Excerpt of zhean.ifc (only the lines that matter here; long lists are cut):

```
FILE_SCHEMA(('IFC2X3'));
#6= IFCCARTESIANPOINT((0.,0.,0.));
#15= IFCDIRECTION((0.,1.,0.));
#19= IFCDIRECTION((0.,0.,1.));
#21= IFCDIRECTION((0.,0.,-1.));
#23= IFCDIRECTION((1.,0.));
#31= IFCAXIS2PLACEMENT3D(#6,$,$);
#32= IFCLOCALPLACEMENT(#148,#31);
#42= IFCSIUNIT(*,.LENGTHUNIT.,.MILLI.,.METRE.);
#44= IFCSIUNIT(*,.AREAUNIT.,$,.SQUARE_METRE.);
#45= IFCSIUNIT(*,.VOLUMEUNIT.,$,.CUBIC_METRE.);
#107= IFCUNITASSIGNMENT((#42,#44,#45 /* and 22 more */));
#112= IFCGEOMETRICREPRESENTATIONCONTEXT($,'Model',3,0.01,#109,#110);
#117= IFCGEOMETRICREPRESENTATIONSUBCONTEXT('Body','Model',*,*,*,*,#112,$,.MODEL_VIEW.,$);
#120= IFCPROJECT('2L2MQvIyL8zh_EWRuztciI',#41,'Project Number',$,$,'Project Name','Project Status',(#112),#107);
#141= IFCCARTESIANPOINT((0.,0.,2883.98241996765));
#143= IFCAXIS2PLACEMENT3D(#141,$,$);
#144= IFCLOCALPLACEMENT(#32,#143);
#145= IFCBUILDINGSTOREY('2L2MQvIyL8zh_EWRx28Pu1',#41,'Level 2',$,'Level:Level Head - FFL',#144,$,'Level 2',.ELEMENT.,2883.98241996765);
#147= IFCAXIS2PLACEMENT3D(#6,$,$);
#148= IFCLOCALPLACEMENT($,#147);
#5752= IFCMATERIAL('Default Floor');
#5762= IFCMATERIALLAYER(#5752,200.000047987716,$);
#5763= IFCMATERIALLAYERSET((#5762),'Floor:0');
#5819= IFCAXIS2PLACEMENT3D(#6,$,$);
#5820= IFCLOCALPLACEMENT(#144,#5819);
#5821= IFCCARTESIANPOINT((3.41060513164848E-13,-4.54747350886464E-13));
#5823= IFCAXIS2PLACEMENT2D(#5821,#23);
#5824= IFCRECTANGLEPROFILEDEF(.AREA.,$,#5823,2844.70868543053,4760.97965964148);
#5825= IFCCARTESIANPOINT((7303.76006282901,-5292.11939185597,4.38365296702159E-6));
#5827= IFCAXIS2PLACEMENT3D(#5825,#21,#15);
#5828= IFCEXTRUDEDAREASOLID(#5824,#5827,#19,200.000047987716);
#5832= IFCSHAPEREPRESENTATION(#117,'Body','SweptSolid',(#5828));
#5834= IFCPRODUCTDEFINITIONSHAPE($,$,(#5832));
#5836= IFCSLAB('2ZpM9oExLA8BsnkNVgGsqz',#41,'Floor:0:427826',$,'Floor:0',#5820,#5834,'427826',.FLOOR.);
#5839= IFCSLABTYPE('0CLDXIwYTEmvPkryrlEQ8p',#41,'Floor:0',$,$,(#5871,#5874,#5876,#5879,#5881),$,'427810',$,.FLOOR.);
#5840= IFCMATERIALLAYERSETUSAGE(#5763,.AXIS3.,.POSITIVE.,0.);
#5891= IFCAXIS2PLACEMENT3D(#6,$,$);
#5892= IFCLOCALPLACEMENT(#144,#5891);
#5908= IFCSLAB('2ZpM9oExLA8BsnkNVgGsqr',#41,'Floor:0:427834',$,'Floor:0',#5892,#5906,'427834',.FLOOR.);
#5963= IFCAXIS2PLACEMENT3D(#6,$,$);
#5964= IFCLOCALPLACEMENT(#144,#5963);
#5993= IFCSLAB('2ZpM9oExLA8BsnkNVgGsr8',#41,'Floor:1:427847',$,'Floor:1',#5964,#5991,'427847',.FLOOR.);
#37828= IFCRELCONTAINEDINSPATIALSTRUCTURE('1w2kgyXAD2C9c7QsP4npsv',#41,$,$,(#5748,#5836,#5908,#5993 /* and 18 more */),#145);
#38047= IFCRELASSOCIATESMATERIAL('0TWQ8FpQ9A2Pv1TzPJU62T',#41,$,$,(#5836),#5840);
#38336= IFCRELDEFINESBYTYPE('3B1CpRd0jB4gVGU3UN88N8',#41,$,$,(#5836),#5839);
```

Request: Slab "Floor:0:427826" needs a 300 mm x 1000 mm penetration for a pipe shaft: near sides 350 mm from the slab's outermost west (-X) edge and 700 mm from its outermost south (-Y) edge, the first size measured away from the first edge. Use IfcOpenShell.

```python
import numpy as np
import ifcopenshell
import ifcopenshell.api.feature
import ifcopenshell.api.geometry
import ifcopenshell.api.root
import ifcopenshell.geom
import ifcopenshell.util.placement
import ifcopenshell.util.representation
import ifcopenshell.util.shape
import ifcopenshell.util.unit

model = ifcopenshell.open("zhean.ifc")
unit_scale = ifcopenshell.util.unit.calculate_unit_scale(model)
settings = ifcopenshell.geom.settings()


def volume(element):
    """Net volume in cubic metres, openings subtracted."""
    shape = ifcopenshell.geom.create_shape(settings, element)
    return ifcopenshell.util.shape.get_volume(shape.geometry)


slab = model.by_id(5836)
before = volume(slab)

# Extent in the slab's own axes, in metres. The edges named are its -X and -Y sides.
slab_shape = ifcopenshell.geom.create_shape(settings, slab)
vertices = ifcopenshell.util.shape.get_vertices(slab_shape.geometry)
x_min, y_min, bottom = vertices.min(axis=0)
top = vertices[:, 2].max()

opening = ifcopenshell.api.root.create_entity(model, ifc_class="IfcOpeningElement", name="Pipe shaft opening")
context = ifcopenshell.util.representation.get_context(model, "Model", "Body", "MODEL_VIEW")
width, depth = 0.3, 1
outline = [(0.0, 0.0), (width, 0.0), (width, depth), (0.0, depth), (0.0, 0.0)]
# Overshoot both faces by 50 mm so the cut is clean.
shape = ifcopenshell.api.geometry.add_slab_representation(
    model, context=context, depth=top - bottom + 0.1, polyline=outline
)
ifcopenshell.api.geometry.assign_representation(model, product=opening, representation=shape)

matrix = ifcopenshell.util.placement.get_local_placement(slab.ObjectPlacement)
matrix[:, 3] = matrix @ np.append(np.array([x_min + 0.35, y_min + 0.7, bottom - 0.05]) / unit_scale, 1.0)
ifcopenshell.api.geometry.edit_object_placement(model, product=opening, matrix=matrix, is_si=False)
ifcopenshell.api.feature.add_feature(model, feature=opening, element=slab)

after = volume(slab)

print(f"slab volume {before:.3f} -> {after:.3f} m3")

model.write("zhean_edited.ifc")
```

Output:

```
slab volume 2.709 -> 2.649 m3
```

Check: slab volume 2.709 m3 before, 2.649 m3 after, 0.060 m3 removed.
